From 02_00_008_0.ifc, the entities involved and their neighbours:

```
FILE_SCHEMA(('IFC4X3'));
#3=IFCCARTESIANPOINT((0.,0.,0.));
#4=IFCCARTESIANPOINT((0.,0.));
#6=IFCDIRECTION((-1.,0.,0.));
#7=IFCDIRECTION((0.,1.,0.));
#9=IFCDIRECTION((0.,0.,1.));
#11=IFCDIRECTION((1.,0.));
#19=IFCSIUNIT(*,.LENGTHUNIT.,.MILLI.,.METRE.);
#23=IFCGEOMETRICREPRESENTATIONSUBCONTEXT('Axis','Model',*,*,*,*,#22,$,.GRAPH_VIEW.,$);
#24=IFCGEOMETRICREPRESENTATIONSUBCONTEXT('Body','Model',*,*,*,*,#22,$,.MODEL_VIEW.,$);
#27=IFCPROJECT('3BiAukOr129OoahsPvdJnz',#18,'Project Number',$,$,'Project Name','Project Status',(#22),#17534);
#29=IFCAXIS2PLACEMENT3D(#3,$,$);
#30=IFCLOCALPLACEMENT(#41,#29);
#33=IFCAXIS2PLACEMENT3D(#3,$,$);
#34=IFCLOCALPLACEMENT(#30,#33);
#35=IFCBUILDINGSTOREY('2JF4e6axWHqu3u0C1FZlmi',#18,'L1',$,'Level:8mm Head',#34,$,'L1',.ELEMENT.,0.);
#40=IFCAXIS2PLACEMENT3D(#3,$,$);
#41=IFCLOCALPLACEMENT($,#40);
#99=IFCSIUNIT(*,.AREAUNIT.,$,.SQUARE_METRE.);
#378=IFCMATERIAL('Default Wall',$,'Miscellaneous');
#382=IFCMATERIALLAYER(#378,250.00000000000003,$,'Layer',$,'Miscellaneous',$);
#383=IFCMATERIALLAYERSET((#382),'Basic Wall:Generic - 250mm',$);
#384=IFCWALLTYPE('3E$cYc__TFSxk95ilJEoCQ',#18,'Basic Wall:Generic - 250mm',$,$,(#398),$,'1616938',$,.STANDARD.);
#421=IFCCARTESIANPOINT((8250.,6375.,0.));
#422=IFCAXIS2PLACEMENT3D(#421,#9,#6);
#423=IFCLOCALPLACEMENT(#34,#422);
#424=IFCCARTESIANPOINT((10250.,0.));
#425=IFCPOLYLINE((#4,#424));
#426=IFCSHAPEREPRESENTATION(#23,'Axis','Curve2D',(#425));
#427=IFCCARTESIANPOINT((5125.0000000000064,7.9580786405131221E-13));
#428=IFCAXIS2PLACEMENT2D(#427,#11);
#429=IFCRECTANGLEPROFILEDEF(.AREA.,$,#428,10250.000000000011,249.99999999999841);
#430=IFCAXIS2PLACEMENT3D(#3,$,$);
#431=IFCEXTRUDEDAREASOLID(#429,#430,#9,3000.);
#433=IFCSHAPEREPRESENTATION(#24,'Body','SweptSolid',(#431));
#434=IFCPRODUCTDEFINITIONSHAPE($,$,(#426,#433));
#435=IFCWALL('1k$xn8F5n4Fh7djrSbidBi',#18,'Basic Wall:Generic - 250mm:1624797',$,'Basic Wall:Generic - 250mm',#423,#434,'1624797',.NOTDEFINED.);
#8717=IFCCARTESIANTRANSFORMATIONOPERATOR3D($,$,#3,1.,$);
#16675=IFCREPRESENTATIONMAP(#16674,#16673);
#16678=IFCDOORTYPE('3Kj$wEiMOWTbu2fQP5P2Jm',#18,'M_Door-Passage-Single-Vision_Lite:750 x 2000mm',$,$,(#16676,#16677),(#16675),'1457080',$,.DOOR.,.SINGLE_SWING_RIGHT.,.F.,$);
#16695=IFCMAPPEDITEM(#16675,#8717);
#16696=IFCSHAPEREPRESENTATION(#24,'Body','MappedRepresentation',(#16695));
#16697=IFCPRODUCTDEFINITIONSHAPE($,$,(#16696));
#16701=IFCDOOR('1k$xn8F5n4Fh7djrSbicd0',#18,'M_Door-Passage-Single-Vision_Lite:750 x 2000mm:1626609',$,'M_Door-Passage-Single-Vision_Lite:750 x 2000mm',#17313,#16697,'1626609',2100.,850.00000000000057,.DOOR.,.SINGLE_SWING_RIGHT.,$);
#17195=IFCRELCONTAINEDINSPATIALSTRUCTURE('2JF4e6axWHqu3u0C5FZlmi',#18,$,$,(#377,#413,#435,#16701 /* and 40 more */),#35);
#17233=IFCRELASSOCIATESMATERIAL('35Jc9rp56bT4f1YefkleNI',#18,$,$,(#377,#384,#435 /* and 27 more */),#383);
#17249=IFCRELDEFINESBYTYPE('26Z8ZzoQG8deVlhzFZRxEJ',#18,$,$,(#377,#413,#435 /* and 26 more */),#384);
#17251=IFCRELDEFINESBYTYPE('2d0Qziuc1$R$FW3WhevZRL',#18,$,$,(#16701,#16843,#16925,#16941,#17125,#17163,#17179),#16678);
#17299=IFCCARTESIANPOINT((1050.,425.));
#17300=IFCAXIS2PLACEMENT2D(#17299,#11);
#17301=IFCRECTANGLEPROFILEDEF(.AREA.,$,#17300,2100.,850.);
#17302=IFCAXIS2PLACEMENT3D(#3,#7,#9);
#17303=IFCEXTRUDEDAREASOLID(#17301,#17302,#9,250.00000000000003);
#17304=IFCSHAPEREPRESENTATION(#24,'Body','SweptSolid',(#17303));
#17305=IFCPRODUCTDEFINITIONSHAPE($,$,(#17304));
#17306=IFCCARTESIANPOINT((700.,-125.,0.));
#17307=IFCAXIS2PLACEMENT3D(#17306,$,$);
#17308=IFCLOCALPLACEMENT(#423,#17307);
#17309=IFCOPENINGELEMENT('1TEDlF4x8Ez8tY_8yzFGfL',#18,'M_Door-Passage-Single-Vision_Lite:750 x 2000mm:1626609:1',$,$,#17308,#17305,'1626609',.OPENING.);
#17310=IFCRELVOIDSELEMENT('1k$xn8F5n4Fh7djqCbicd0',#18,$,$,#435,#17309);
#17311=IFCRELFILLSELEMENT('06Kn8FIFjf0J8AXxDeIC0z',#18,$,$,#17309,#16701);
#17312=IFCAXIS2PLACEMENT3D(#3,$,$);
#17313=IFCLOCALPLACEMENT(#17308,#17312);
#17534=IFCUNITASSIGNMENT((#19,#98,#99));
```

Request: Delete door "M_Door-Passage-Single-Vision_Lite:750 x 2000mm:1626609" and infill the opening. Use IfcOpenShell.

```python
import ifcopenshell
import ifcopenshell.api.feature
import ifcopenshell.api.root
import ifcopenshell.geom
import ifcopenshell.util.shape

model = ifcopenshell.open("02_00_008_0.ifc")
settings = ifcopenshell.geom.settings()


def volume(element):
    """Net volume in cubic metres, openings subtracted."""
    shape = ifcopenshell.geom.create_shape(settings, element)
    return ifcopenshell.util.shape.get_volume(shape.geometry)


door = model.by_guid("1k$xn8F5n4Fh7djrSbicd0")
opening = door.FillsVoids[0].RelatingOpeningElement
wall = opening.VoidsElements[0].RelatingBuildingElement
before = volume(wall)

ifcopenshell.api.root.remove_product(model, product=door)
ifcopenshell.api.feature.remove_feature(model, feature=opening)

after = volume(wall)

print(f"wall volume {before:.3f} -> {after:.3f} m3")

model.write("02_00_008_0_rev.ifc")
```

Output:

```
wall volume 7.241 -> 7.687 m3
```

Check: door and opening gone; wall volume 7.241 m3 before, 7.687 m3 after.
